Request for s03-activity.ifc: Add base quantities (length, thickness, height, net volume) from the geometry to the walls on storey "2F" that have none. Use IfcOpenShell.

First a look at what the model holds.

```python
import ifcopenshell
import ifcopenshell.util.element
import ifcopenshell.util.unit

model = ifcopenshell.open("s03-activity.ifc")
print(model.schema)
for unit_type in ("LENGTHUNIT", "AREAUNIT", "VOLUMEUNIT"):
    print(unit_type, ifcopenshell.util.unit.calculate_unit_scale(model, unit_type))
storey = next(s for s in model.by_type("IfcBuildingStorey") if s.Name == "2F")
walls = [e for e in ifcopenshell.util.element.get_decomposition(storey) if e.is_a("IfcWall")]
for e in sorted(walls, key=lambda e: e.id()):
    print(e.id(), e.is_a(), e.Name, list(ifcopenshell.util.element.get_psets(e, qtos_only=True)), sep=" | ")
```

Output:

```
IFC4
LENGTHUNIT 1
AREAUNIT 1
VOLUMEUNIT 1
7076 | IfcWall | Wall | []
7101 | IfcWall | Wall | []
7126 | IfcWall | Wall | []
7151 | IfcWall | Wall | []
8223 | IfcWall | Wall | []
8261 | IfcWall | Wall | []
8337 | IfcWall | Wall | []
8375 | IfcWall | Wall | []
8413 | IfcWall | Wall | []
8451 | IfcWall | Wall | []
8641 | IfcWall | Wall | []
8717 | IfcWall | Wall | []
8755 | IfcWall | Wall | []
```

```python
import ifcopenshell
import ifcopenshell.api.pset
import ifcopenshell.geom
import ifcopenshell.util.element
import ifcopenshell.util.shape
import ifcopenshell.util.unit

model = ifcopenshell.open("s03-activity.ifc")
unit_scale = ifcopenshell.util.unit.calculate_unit_scale(model)
volume_scale = ifcopenshell.util.unit.calculate_unit_scale(model, "VOLUMEUNIT")
settings = ifcopenshell.geom.settings()

storey = next(s for s in model.by_type("IfcBuildingStorey") if s.Name == "2F")
walls = [e for e in ifcopenshell.util.element.get_decomposition(storey) if e.is_a("IfcWall")]

for e in sorted(walls, key=lambda e: e.id()):
    if ifcopenshell.util.element.get_psets(e, qtos_only=True, should_inherit=False):
        continue
    # Geometry comes back in metres, in the element's own axes.
    shape = ifcopenshell.geom.create_shape(settings, e)
    values = {
        "Length": ifcopenshell.util.shape.get_x(shape.geometry) / unit_scale,
        "Width": ifcopenshell.util.shape.get_y(shape.geometry) / unit_scale,
        "Height": ifcopenshell.util.shape.get_z(shape.geometry) / unit_scale,
        "NetVolume": ifcopenshell.util.shape.get_volume(shape.geometry) / volume_scale,
    }
    qto = ifcopenshell.api.pset.add_qto(model, product=e, name="Qto_WallBaseQuantities")
    ifcopenshell.api.pset.edit_qto(model, qto=qto, properties=values)
    print(e.id(), {k: round(v, 3) for k, v in values.items()})

model.write("s03-activity_edited.ifc")
```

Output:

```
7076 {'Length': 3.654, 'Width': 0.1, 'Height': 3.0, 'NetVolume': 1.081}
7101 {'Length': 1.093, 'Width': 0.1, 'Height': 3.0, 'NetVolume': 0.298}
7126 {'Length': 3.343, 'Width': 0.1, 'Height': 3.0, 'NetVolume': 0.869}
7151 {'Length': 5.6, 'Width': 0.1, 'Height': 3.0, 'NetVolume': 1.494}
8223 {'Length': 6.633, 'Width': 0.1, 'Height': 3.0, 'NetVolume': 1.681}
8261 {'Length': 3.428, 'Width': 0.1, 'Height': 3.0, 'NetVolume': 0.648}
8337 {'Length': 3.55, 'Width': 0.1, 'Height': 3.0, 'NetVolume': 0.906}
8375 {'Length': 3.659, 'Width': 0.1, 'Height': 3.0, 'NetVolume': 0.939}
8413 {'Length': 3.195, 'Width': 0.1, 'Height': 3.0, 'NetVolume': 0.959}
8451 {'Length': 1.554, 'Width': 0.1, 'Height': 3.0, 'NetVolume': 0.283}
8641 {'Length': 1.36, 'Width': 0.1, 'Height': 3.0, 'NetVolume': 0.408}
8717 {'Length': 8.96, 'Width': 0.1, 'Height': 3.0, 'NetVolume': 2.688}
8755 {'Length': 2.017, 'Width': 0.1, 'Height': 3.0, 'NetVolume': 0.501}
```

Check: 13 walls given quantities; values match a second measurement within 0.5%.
